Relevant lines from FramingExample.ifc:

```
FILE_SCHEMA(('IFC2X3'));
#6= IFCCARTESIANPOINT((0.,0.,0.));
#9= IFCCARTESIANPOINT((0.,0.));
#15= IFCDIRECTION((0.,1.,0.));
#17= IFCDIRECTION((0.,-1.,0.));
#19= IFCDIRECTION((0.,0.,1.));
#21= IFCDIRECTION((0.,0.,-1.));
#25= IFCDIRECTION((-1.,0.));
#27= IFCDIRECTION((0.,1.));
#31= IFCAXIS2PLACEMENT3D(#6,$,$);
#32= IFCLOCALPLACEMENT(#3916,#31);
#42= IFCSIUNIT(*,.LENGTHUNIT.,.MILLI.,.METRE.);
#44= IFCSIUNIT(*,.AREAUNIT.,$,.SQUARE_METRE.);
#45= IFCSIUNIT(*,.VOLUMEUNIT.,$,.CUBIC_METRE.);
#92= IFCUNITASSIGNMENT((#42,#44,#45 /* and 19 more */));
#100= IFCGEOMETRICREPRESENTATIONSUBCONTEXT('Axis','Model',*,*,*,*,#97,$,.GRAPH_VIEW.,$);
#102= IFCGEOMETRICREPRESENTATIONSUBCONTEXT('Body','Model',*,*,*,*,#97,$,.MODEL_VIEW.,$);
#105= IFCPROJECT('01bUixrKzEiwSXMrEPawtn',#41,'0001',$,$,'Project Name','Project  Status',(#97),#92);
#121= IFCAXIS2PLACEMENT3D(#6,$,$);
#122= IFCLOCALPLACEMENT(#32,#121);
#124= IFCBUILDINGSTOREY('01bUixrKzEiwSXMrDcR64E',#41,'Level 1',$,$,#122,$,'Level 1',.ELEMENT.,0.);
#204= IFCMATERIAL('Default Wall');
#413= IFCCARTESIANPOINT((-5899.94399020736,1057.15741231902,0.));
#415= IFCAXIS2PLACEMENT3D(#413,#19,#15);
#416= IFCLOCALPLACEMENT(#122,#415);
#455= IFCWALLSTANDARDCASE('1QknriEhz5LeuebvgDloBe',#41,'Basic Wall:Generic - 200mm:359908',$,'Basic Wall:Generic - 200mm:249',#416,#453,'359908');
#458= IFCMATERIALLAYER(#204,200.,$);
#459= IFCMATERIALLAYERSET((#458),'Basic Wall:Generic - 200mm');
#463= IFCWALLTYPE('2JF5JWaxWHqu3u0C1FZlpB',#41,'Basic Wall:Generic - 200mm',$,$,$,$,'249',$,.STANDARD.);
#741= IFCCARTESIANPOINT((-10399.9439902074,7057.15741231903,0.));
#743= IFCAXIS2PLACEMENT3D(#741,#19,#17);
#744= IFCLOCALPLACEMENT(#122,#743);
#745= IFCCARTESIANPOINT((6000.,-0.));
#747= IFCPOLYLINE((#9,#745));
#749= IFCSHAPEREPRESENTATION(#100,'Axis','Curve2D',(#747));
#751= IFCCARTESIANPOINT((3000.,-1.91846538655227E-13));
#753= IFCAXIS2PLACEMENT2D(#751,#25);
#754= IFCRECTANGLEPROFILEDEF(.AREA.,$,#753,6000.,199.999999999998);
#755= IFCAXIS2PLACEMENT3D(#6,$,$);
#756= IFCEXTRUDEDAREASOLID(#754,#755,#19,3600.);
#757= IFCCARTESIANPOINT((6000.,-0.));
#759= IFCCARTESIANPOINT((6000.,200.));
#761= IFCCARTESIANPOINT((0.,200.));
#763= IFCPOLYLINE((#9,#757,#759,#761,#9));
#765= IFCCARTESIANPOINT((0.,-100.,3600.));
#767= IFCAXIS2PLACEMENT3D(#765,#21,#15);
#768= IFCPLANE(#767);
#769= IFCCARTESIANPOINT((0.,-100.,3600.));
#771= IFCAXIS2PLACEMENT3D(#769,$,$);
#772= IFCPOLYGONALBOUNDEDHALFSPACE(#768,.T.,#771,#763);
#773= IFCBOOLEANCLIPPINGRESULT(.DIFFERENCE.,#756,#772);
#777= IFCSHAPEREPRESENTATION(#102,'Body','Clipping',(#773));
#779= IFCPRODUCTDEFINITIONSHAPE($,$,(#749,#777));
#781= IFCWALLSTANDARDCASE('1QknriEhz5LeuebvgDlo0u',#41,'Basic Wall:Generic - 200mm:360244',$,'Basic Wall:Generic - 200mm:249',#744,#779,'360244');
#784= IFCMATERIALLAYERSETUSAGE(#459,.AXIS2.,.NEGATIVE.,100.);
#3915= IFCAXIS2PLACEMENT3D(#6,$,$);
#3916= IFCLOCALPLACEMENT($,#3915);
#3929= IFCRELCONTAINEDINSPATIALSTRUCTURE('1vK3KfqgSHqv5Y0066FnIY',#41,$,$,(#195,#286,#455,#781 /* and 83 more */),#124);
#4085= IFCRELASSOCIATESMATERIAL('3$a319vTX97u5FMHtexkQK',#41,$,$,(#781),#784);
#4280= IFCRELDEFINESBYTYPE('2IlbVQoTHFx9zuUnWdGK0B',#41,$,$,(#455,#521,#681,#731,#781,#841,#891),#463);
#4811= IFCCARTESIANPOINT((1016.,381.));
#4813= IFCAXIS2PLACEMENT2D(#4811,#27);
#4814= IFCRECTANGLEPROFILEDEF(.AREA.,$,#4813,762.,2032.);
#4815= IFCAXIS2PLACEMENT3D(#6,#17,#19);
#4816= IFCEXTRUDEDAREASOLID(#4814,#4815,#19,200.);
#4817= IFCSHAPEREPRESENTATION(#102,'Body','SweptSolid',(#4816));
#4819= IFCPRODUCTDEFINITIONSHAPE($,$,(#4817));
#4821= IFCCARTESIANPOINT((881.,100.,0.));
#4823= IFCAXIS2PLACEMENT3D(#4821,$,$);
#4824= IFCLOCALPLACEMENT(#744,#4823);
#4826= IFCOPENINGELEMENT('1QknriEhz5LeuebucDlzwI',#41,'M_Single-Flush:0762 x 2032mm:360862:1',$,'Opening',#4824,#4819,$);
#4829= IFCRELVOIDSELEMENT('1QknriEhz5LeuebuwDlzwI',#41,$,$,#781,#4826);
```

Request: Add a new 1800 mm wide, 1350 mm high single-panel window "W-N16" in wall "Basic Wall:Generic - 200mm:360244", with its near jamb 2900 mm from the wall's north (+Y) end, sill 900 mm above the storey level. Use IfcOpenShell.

```python
import numpy as np
import ifcopenshell
import ifcopenshell.api.feature
import ifcopenshell.api.geometry
import ifcopenshell.api.root
import ifcopenshell.api.spatial
import ifcopenshell.api.type
import ifcopenshell.geom
import ifcopenshell.util.element
import ifcopenshell.util.placement
import ifcopenshell.util.representation
import ifcopenshell.util.shape
import ifcopenshell.util.unit

model = ifcopenshell.open("FramingExample.ifc")
unit_scale = ifcopenshell.util.unit.calculate_unit_scale(model)
settings = ifcopenshell.geom.settings()


def volume(element):
    """Net volume in cubic metres, openings subtracted."""
    shape = ifcopenshell.geom.create_shape(settings, element)
    return ifcopenshell.util.shape.get_volume(shape.geometry)


wall = model.by_guid("1QknriEhz5LeuebvgDlo0u")
storey = ifcopenshell.util.element.get_container(wall, ifc_class="IfcBuildingStorey")
context = ifcopenshell.util.representation.get_context(model, "Model", "Body", "MODEL_VIEW")
before = volume(wall)

width, height, from_end, sill = 1.8, 1.35, 2.9, 0.9  # metres

# The wall runs along its own X axis, and the end named is its -X end.
wall_shape = ifcopenshell.geom.create_shape(settings, wall)
x, y, z = ifcopenshell.util.shape.get_vertices(wall_shape.geometry).T
start = x.min() + from_end
face, thickness = float(y.min()), float(y.max() - y.min())
wall_matrix = ifcopenshell.util.placement.get_local_placement(wall.ObjectPlacement)
level = ifcopenshell.util.placement.get_local_placement(storey.ObjectPlacement)[2, 3]


def in_wall(x, y):
    """Placement at x, y metres in the wall's axes, at sill height."""
    matrix = wall_matrix.copy()
    matrix[:, 3] = wall_matrix @ np.array([x / unit_scale, y / unit_scale, 0.0, 1.0])
    matrix[2, 3] = level + sill / unit_scale
    return matrix


# Opening: a box that overshoots both wall faces by 50 mm.
opening = ifcopenshell.api.root.create_entity(model, ifc_class="IfcOpeningElement")
box = ifcopenshell.api.geometry.add_wall_representation(
    model, context=context, length=width, height=height, thickness=thickness + 0.1
)
ifcopenshell.api.geometry.assign_representation(model, product=opening, representation=box)
ifcopenshell.api.geometry.edit_object_placement(model, product=opening, matrix=in_wall(start, face - 0.05), is_si=False)
ifcopenshell.api.feature.add_feature(model, feature=opening, element=wall)

window = ifcopenshell.api.root.create_entity(model, ifc_class="IfcWindow", name="W-N16")
window.OverallWidth, window.OverallHeight = width / unit_scale, height / unit_scale
body = ifcopenshell.api.geometry.add_window_representation(
    model,
    context=context,
    overall_width=window.OverallWidth,
    overall_height=window.OverallHeight,
    partition_type="SINGLE_PANEL",
)
ifcopenshell.api.geometry.assign_representation(model, product=window, representation=body)
ifcopenshell.api.spatial.assign_container(model, products=[window], relating_structure=storey)
fills = ifcopenshell.api.feature.add_filling(model, opening=opening, element=window)
fills.OwnerHistory = window.OwnerHistory  # required in IFC2X3

# IFC2X3 keeps the operation on the window style.
style = ifcopenshell.api.root.create_entity(model, ifc_class="IfcWindowStyle", name="W-N16")
style.OperationType, style.ConstructionType = "SINGLE_PANEL", "NOTDEFINED"
style.ParameterTakesPrecedence = style.Sizeable = False
ifcopenshell.api.type.assign_type(model, related_objects=[window], relating_type=style)

# Centre the window in the wall's thickness.
ifcopenshell.api.geometry.edit_object_placement(model, product=window, matrix=in_wall(start, face), is_si=False)
window_shape = ifcopenshell.geom.create_shape(settings, window)
depth = ifcopenshell.util.shape.get_vertices(window_shape.geometry)[:, 1]
offset = face + thickness / 2 - (depth.min() + depth.max()) / 2
ifcopenshell.api.geometry.edit_object_placement(model, product=window, matrix=in_wall(start, offset), is_si=False)

after = volume(wall)

print(f"wall volume {before:.3f} -> {after:.3f} m3")

model.write("FramingExample_edited.ifc")
```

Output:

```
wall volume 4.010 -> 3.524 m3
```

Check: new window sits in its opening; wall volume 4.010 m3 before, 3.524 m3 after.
